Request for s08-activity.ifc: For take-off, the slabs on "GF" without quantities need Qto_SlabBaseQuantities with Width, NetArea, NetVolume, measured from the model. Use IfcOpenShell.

First a look at what the model holds.

```python
import ifcopenshell
import ifcopenshell.util.element
import ifcopenshell.util.unit

model = ifcopenshell.open("s08-activity.ifc")
print(model.schema)
for unit_type in ("LENGTHUNIT", "AREAUNIT", "VOLUMEUNIT"):
    print(unit_type, ifcopenshell.util.unit.calculate_unit_scale(model, unit_type))
storey = next(s for s in model.by_type("IfcBuildingStorey") if s.Name == "GF")
slabs = [e for e in ifcopenshell.util.element.get_decomposition(storey) if e.is_a("IfcSlab")]
for e in sorted(slabs, key=lambda e: e.id()):
    print(e.id(), e.is_a(), e.Name, list(ifcopenshell.util.element.get_psets(e, qtos_only=True)), sep=" | ")
```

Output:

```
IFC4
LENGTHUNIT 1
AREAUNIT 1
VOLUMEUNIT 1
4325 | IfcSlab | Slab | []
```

```python
import ifcopenshell
import ifcopenshell.api.pset
import ifcopenshell.geom
import ifcopenshell.util.element
import ifcopenshell.util.shape
import ifcopenshell.util.unit

model = ifcopenshell.open("s08-activity.ifc")
unit_scale = ifcopenshell.util.unit.calculate_unit_scale(model)
area_scale = ifcopenshell.util.unit.calculate_unit_scale(model, "AREAUNIT")
volume_scale = ifcopenshell.util.unit.calculate_unit_scale(model, "VOLUMEUNIT")
settings = ifcopenshell.geom.settings()

storey = next(s for s in model.by_type("IfcBuildingStorey") if s.Name == "GF")
slabs = [e for e in ifcopenshell.util.element.get_decomposition(storey) if e.is_a("IfcSlab")]

for e in sorted(slabs, key=lambda e: e.id()):
    if ifcopenshell.util.element.get_psets(e, qtos_only=True, should_inherit=False):
        continue
    # Geometry comes back in metres, in the element's own axes.
    shape = ifcopenshell.geom.create_shape(settings, e)
    values = {
        "Width": ifcopenshell.util.shape.get_z(shape.geometry) / unit_scale,
        "NetArea": ifcopenshell.util.shape.get_footprint_area(shape.geometry) / area_scale,
        "NetVolume": ifcopenshell.util.shape.get_volume(shape.geometry) / volume_scale,
    }
    qto = ifcopenshell.api.pset.add_qto(model, product=e, name="Qto_SlabBaseQuantities")
    ifcopenshell.api.pset.edit_qto(model, qto=qto, properties=values)
    print(e.id(), {k: round(v, 3) for k, v in values.items()})

model.write("s08-activity_rev.ifc")
```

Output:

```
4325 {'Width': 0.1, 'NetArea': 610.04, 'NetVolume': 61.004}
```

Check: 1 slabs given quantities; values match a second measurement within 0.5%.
